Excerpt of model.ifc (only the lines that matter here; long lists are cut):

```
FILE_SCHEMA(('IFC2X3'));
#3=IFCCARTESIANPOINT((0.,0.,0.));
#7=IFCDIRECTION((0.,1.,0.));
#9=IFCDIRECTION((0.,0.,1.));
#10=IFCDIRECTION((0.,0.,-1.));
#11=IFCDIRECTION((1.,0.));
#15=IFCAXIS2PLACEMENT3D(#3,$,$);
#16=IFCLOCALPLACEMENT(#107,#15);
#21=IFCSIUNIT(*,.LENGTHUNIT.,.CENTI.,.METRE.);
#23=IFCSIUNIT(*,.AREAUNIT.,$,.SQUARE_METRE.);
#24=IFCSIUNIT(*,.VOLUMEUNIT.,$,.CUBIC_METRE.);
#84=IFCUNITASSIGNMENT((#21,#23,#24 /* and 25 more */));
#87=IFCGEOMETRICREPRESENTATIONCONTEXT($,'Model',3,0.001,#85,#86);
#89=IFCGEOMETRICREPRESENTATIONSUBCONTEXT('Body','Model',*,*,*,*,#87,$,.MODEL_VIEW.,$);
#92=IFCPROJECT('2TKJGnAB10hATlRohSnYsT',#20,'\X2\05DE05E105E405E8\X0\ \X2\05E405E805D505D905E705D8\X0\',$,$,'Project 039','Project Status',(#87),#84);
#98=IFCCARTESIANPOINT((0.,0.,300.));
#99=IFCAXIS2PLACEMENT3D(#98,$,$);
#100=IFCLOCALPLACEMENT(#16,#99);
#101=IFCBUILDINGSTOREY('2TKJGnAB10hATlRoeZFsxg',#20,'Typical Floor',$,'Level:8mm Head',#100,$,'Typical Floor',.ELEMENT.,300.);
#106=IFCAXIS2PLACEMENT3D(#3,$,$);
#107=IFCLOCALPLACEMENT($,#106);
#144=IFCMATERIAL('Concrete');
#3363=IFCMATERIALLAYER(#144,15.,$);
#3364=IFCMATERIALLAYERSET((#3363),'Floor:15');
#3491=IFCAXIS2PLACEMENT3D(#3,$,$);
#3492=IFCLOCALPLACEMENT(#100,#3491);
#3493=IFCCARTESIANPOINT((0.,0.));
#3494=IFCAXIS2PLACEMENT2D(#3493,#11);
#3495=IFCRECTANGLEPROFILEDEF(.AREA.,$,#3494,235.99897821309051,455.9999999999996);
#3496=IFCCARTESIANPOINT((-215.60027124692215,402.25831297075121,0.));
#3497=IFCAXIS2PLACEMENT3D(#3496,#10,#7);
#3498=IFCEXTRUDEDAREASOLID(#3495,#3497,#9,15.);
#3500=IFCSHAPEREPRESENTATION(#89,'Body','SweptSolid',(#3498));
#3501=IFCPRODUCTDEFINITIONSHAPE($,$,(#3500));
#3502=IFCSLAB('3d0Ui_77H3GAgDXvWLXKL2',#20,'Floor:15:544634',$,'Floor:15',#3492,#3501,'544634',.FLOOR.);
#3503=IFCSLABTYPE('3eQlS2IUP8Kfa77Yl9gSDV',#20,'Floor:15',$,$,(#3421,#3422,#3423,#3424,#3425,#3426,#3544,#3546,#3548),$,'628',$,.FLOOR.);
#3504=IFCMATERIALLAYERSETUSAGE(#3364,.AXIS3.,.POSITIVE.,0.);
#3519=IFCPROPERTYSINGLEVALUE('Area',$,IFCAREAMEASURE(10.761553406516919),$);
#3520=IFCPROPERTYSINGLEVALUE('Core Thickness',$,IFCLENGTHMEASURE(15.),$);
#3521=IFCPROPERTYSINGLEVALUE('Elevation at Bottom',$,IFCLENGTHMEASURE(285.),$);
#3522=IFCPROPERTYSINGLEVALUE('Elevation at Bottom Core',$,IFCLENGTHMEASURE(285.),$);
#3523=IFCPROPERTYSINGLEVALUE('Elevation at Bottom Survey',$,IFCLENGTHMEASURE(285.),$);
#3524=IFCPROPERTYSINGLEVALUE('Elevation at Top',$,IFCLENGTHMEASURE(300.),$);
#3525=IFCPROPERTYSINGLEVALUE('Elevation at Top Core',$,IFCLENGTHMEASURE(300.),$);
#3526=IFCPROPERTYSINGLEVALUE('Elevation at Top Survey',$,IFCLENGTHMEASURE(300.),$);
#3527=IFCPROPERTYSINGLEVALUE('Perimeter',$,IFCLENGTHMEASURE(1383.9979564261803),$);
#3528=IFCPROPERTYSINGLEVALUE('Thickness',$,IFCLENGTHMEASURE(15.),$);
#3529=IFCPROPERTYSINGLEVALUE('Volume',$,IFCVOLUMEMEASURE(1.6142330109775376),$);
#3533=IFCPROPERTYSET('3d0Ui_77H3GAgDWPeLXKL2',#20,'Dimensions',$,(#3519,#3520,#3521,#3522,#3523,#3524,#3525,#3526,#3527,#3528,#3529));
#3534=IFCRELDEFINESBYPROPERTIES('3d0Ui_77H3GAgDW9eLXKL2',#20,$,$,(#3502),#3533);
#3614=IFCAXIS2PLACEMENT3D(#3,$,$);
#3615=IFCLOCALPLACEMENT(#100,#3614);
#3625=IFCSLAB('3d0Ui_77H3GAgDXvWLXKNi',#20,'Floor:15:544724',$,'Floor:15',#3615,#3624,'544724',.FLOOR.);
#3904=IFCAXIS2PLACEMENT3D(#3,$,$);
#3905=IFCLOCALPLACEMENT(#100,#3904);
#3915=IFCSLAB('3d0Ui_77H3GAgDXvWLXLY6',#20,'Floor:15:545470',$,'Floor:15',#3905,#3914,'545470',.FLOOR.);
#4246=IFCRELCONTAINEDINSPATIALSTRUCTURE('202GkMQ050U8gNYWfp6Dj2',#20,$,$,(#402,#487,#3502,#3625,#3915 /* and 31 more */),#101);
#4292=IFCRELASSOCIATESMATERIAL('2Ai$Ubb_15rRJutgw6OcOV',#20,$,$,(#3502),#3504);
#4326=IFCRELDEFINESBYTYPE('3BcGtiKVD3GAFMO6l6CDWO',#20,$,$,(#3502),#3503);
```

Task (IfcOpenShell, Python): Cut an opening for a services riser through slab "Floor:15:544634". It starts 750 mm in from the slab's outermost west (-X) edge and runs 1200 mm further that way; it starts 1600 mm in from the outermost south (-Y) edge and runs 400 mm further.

```python
import numpy as np
import ifcopenshell
import ifcopenshell.api.feature
import ifcopenshell.api.geometry
import ifcopenshell.api.pset
import ifcopenshell.api.root
import ifcopenshell.geom
import ifcopenshell.util.element
import ifcopenshell.util.placement
import ifcopenshell.util.representation
import ifcopenshell.util.shape
import ifcopenshell.util.unit

model = ifcopenshell.open("model.ifc")
unit_scale = ifcopenshell.util.unit.calculate_unit_scale(model)
area_scale = ifcopenshell.util.unit.calculate_unit_scale(model, "AREAUNIT")
volume_scale = ifcopenshell.util.unit.calculate_unit_scale(model, "VOLUMEUNIT")
settings = ifcopenshell.geom.settings()


def volume(element):
    """Net volume in cubic metres, openings subtracted."""
    shape = ifcopenshell.geom.create_shape(settings, element)
    return ifcopenshell.util.shape.get_volume(shape.geometry)


slab = model.by_guid("3d0Ui_77H3GAgDXvWLXKL2")
before = volume(slab)

# Extent in the slab's own axes, in metres. The edges named are its -X and -Y sides.
slab_shape = ifcopenshell.geom.create_shape(settings, slab)
vertices = ifcopenshell.util.shape.get_vertices(slab_shape.geometry)
x_min, y_min, bottom = vertices.min(axis=0)
top = vertices[:, 2].max()

opening = ifcopenshell.api.root.create_entity(model, ifc_class="IfcOpeningElement", name="Services riser opening")
context = ifcopenshell.util.representation.get_context(model, "Model", "Body", "MODEL_VIEW")
width, depth = 1.2, 0.4
outline = [(0.0, 0.0), (width, 0.0), (width, depth), (0.0, depth), (0.0, 0.0)]
# Overshoot both faces by 50 mm so the cut is clean.
shape = ifcopenshell.api.geometry.add_slab_representation(
    model, context=context, depth=top - bottom + 0.1, polyline=outline
)
ifcopenshell.api.geometry.assign_representation(model, product=opening, representation=shape)

matrix = ifcopenshell.util.placement.get_local_placement(slab.ObjectPlacement)
matrix[:, 3] = matrix @ np.append(np.array([x_min + 0.75, y_min + 1.6, bottom - 0.05]) / unit_scale, 1.0)
ifcopenshell.api.geometry.edit_object_placement(model, product=opening, matrix=matrix, is_si=False)
ifcopenshell.api.feature.add_feature(model, feature=opening, element=slab)

after = volume(slab)

# Update the slab's stored quantities.
pset = model.by_id(ifcopenshell.util.element.get_pset(slab, "Dimensions", should_inherit=False)["id"])
ifcopenshell.api.pset.edit_pset(model, pset=pset, properties={
    "Area": model.create_entity("IfcAreaMeasure", after / (top - bottom) / area_scale),
    "Volume": model.create_entity("IfcVolumeMeasure", after / volume_scale),
})

print(f"slab volume {before:.3f} -> {after:.3f} m3")

model.write("model_updated.ifc")
```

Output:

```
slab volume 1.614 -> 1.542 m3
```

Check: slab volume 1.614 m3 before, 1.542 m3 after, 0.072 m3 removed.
